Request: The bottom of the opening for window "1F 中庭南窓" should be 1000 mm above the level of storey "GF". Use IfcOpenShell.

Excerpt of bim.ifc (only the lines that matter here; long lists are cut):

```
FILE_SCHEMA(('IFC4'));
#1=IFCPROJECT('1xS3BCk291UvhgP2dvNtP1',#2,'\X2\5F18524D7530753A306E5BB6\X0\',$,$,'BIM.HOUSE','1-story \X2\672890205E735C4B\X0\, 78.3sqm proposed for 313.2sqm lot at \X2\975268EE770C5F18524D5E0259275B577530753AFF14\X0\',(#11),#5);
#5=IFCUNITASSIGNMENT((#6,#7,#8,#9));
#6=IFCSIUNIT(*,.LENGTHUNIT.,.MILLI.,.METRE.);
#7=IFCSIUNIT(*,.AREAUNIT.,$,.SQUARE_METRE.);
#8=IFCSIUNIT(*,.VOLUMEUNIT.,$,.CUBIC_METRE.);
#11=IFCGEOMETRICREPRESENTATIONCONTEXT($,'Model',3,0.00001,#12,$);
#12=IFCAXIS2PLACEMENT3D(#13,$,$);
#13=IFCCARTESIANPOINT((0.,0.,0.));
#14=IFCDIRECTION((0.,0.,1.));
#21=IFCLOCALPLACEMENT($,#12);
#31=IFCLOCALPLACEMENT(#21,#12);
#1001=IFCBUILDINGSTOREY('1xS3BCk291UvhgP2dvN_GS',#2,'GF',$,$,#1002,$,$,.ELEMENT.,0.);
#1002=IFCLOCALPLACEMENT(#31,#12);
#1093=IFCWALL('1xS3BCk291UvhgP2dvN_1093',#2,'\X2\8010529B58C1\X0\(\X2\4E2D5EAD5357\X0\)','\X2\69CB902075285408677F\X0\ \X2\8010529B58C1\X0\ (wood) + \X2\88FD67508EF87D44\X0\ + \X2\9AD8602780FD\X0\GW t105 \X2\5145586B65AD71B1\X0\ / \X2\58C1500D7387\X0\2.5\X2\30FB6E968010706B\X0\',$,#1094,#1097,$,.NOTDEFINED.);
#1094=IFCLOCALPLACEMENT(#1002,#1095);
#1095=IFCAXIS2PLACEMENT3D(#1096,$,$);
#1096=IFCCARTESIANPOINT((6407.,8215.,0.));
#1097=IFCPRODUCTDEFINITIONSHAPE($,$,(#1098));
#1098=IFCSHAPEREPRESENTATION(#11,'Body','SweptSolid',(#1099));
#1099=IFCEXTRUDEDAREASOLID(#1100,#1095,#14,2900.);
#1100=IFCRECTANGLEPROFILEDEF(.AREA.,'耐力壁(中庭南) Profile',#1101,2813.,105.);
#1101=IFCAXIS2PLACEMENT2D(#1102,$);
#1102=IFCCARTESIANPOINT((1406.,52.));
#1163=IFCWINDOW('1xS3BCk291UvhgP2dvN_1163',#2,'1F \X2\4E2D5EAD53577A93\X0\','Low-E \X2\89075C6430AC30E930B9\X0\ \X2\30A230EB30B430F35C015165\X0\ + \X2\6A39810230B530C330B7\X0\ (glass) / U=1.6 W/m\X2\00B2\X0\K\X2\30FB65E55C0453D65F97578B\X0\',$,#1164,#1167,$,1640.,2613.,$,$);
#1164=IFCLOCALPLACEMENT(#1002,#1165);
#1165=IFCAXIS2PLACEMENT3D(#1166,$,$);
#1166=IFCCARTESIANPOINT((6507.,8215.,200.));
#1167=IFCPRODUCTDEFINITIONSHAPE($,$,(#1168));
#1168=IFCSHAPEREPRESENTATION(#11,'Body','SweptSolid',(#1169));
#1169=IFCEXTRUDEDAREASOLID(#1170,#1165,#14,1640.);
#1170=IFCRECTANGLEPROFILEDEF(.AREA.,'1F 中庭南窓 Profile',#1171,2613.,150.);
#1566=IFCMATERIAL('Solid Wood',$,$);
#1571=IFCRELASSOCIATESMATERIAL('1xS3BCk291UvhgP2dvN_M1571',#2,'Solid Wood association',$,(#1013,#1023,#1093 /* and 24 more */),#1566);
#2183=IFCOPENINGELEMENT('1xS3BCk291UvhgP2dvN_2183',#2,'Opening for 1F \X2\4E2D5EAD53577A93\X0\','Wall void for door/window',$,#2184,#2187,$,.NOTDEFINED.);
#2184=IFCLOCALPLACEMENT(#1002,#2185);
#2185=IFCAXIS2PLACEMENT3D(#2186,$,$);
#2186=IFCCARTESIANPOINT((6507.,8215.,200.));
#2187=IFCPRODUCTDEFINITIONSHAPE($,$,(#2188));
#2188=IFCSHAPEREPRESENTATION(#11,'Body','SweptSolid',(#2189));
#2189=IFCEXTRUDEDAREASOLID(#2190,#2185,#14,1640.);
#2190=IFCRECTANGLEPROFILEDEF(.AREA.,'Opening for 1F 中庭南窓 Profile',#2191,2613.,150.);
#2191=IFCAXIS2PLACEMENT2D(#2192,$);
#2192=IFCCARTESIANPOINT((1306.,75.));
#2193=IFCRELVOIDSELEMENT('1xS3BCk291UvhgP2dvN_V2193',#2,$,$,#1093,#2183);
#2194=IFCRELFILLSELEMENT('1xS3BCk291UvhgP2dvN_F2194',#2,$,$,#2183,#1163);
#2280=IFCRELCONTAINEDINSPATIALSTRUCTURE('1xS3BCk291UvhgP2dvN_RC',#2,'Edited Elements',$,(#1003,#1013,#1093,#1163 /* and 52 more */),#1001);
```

```python
import numpy as np
import ifcopenshell
import ifcopenshell.api.geometry
import ifcopenshell.geom
import ifcopenshell.util.element
import ifcopenshell.util.placement
import ifcopenshell.util.shape
import ifcopenshell.util.unit

model = ifcopenshell.open("bim.ifc")
unit_scale = ifcopenshell.util.unit.calculate_unit_scale(model)

window = model.by_guid("1xS3BCk291UvhgP2dvN_1163")
opening = window.FillsVoids[0].RelatingOpeningElement
storey = ifcopenshell.util.element.get_container(window, ifc_class="IfcBuildingStorey")
level = ifcopenshell.util.placement.get_local_placement(storey.ObjectPlacement)[2, 3]

# The opening's origin need not be at the sill, so measure its lowest point.
shape = ifcopenshell.geom.create_shape(ifcopenshell.geom.settings(), opening)
bottom = ifcopenshell.util.shape.get_shape_bottom_elevation(shape, shape.geometry) / unit_scale
dz = level + 1000.0 - bottom

shift = np.array([0.0, 0.0, dz])
# The window is not placed relative to its opening, so move both.
for product in (opening, window):
    matrix = ifcopenshell.util.placement.get_local_placement(product.ObjectPlacement)
    matrix[:3, 3] += shift
    ifcopenshell.api.geometry.edit_object_placement(model, product=product, matrix=matrix, is_si=False)

print(f"moved by {dz * unit_scale:+.3f} m")

model.write("bim-out.ifc")
```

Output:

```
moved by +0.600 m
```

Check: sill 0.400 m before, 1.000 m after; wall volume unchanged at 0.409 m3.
